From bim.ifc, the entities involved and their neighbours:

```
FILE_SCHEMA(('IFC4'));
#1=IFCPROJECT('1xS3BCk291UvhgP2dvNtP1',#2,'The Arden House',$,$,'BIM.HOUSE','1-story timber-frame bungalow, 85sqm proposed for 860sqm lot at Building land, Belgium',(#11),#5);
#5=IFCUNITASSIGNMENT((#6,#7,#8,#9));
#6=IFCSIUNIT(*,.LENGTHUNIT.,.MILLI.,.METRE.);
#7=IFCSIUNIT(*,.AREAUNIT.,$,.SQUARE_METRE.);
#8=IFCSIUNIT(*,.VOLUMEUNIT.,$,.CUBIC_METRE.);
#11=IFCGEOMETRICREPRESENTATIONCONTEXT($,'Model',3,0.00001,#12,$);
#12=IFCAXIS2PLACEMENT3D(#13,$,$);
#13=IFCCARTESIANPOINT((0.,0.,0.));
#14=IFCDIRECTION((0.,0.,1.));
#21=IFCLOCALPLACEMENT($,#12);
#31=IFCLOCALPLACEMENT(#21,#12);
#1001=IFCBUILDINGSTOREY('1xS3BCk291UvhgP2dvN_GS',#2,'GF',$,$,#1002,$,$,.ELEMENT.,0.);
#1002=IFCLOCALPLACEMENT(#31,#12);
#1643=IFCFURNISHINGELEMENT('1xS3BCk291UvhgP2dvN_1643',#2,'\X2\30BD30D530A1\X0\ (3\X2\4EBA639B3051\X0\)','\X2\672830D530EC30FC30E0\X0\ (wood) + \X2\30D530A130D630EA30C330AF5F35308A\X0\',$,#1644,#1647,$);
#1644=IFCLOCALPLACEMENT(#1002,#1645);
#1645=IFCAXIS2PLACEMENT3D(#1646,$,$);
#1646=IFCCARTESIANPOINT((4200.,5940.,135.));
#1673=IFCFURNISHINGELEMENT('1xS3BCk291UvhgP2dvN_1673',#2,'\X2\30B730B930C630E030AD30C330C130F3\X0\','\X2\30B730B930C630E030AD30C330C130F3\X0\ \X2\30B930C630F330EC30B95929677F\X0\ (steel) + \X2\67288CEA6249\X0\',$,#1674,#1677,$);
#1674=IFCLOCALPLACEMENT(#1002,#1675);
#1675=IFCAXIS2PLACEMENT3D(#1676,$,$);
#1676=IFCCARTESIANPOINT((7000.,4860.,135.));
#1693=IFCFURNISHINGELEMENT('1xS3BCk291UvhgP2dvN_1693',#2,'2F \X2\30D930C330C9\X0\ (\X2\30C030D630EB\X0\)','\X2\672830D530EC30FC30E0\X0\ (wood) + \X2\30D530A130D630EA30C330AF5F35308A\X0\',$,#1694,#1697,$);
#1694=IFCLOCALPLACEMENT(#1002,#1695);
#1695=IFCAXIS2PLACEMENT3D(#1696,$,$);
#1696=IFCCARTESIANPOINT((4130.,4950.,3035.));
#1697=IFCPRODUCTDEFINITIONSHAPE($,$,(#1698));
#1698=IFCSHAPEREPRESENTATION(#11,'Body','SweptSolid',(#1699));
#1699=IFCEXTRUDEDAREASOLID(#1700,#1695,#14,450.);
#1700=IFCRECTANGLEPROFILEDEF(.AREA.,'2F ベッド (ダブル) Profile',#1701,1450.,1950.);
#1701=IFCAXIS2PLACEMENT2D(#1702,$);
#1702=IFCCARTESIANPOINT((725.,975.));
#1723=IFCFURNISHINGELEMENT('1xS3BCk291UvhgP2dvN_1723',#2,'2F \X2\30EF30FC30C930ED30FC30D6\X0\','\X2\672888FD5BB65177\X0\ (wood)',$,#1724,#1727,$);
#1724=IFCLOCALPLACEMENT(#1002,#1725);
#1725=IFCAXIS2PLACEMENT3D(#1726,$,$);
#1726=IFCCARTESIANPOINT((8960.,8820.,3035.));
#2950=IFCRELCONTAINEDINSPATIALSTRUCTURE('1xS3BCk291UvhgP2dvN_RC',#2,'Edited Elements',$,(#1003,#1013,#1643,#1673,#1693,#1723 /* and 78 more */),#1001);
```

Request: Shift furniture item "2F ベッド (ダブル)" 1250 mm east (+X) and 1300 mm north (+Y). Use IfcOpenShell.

```python
import ifcopenshell
import ifcopenshell.api.geometry
import ifcopenshell.util.placement
import ifcopenshell.util.unit

model = ifcopenshell.open("bim.ifc")
unit_scale = ifcopenshell.util.unit.calculate_unit_scale(model)

item = model.by_guid("1xS3BCk291UvhgP2dvN_1693")
matrix = ifcopenshell.util.placement.get_local_placement(item.ObjectPlacement)
matrix[0, 3] += 1.25 / unit_scale
matrix[1, 3] += 1.3 / unit_scale
ifcopenshell.api.geometry.edit_object_placement(model, product=item, matrix=matrix, is_si=False)

print(ifcopenshell.util.placement.get_local_placement(item.ObjectPlacement).round(3) + 0.0)

model.write("bim_updated.ifc")
```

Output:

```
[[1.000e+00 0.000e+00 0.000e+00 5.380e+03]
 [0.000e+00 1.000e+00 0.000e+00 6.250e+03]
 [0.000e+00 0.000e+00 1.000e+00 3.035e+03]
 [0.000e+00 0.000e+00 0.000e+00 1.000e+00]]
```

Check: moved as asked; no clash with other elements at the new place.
